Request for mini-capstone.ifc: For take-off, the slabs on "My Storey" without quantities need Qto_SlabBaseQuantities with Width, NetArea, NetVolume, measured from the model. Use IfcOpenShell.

First a look at what the model holds.

```python
import ifcopenshell
import ifcopenshell.util.element
import ifcopenshell.util.unit

model = ifcopenshell.open("mini-capstone.ifc")
print(model.schema)
for unit_type in ("LENGTHUNIT", "AREAUNIT", "VOLUMEUNIT"):
    print(unit_type, ifcopenshell.util.unit.calculate_unit_scale(model, unit_type))
storey = next(s for s in model.by_type("IfcBuildingStorey") if s.Name == "My Storey")
slabs = [e for e in ifcopenshell.util.element.get_decomposition(storey) if e.is_a("IfcSlab")]
for e in sorted(slabs, key=lambda e: e.id()):
    print(e.id(), e.is_a(), e.Name, list(ifcopenshell.util.element.get_psets(e, qtos_only=True)), sep=" | ")
```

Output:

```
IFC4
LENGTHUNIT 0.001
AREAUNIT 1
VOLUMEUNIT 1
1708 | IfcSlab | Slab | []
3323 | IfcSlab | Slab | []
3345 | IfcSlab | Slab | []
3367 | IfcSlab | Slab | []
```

```python
import ifcopenshell
import ifcopenshell.api.pset
import ifcopenshell.geom
import ifcopenshell.util.element
import ifcopenshell.util.shape
import ifcopenshell.util.unit

model = ifcopenshell.open("mini-capstone.ifc")
unit_scale = ifcopenshell.util.unit.calculate_unit_scale(model)
area_scale = ifcopenshell.util.unit.calculate_unit_scale(model, "AREAUNIT")
volume_scale = ifcopenshell.util.unit.calculate_unit_scale(model, "VOLUMEUNIT")
settings = ifcopenshell.geom.settings()

storey = next(s for s in model.by_type("IfcBuildingStorey") if s.Name == "My Storey")
slabs = [e for e in ifcopenshell.util.element.get_decomposition(storey) if e.is_a("IfcSlab")]

for e in sorted(slabs, key=lambda e: e.id()):
    if ifcopenshell.util.element.get_psets(e, qtos_only=True, should_inherit=False):
        continue
    # Geometry comes back in metres, in the element's own axes.
    shape = ifcopenshell.geom.create_shape(settings, e)
    values = {
        "Width": ifcopenshell.util.shape.get_z(shape.geometry) / unit_scale,
        "NetArea": ifcopenshell.util.shape.get_footprint_area(shape.geometry) / area_scale,
        "NetVolume": ifcopenshell.util.shape.get_volume(shape.geometry) / volume_scale,
    }
    qto = ifcopenshell.api.pset.add_qto(model, product=e, name="Qto_SlabBaseQuantities")
    ifcopenshell.api.pset.edit_qto(model, qto=qto, properties=values)
    print(e.id(), {k: round(v, 3) for k, v in values.items()})

model.write("mini-capstone_rev.ifc")
```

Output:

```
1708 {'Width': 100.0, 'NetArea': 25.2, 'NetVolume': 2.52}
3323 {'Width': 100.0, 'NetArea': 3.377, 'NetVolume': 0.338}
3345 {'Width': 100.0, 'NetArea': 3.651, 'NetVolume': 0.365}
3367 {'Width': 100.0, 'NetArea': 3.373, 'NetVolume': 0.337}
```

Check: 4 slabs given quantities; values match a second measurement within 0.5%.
